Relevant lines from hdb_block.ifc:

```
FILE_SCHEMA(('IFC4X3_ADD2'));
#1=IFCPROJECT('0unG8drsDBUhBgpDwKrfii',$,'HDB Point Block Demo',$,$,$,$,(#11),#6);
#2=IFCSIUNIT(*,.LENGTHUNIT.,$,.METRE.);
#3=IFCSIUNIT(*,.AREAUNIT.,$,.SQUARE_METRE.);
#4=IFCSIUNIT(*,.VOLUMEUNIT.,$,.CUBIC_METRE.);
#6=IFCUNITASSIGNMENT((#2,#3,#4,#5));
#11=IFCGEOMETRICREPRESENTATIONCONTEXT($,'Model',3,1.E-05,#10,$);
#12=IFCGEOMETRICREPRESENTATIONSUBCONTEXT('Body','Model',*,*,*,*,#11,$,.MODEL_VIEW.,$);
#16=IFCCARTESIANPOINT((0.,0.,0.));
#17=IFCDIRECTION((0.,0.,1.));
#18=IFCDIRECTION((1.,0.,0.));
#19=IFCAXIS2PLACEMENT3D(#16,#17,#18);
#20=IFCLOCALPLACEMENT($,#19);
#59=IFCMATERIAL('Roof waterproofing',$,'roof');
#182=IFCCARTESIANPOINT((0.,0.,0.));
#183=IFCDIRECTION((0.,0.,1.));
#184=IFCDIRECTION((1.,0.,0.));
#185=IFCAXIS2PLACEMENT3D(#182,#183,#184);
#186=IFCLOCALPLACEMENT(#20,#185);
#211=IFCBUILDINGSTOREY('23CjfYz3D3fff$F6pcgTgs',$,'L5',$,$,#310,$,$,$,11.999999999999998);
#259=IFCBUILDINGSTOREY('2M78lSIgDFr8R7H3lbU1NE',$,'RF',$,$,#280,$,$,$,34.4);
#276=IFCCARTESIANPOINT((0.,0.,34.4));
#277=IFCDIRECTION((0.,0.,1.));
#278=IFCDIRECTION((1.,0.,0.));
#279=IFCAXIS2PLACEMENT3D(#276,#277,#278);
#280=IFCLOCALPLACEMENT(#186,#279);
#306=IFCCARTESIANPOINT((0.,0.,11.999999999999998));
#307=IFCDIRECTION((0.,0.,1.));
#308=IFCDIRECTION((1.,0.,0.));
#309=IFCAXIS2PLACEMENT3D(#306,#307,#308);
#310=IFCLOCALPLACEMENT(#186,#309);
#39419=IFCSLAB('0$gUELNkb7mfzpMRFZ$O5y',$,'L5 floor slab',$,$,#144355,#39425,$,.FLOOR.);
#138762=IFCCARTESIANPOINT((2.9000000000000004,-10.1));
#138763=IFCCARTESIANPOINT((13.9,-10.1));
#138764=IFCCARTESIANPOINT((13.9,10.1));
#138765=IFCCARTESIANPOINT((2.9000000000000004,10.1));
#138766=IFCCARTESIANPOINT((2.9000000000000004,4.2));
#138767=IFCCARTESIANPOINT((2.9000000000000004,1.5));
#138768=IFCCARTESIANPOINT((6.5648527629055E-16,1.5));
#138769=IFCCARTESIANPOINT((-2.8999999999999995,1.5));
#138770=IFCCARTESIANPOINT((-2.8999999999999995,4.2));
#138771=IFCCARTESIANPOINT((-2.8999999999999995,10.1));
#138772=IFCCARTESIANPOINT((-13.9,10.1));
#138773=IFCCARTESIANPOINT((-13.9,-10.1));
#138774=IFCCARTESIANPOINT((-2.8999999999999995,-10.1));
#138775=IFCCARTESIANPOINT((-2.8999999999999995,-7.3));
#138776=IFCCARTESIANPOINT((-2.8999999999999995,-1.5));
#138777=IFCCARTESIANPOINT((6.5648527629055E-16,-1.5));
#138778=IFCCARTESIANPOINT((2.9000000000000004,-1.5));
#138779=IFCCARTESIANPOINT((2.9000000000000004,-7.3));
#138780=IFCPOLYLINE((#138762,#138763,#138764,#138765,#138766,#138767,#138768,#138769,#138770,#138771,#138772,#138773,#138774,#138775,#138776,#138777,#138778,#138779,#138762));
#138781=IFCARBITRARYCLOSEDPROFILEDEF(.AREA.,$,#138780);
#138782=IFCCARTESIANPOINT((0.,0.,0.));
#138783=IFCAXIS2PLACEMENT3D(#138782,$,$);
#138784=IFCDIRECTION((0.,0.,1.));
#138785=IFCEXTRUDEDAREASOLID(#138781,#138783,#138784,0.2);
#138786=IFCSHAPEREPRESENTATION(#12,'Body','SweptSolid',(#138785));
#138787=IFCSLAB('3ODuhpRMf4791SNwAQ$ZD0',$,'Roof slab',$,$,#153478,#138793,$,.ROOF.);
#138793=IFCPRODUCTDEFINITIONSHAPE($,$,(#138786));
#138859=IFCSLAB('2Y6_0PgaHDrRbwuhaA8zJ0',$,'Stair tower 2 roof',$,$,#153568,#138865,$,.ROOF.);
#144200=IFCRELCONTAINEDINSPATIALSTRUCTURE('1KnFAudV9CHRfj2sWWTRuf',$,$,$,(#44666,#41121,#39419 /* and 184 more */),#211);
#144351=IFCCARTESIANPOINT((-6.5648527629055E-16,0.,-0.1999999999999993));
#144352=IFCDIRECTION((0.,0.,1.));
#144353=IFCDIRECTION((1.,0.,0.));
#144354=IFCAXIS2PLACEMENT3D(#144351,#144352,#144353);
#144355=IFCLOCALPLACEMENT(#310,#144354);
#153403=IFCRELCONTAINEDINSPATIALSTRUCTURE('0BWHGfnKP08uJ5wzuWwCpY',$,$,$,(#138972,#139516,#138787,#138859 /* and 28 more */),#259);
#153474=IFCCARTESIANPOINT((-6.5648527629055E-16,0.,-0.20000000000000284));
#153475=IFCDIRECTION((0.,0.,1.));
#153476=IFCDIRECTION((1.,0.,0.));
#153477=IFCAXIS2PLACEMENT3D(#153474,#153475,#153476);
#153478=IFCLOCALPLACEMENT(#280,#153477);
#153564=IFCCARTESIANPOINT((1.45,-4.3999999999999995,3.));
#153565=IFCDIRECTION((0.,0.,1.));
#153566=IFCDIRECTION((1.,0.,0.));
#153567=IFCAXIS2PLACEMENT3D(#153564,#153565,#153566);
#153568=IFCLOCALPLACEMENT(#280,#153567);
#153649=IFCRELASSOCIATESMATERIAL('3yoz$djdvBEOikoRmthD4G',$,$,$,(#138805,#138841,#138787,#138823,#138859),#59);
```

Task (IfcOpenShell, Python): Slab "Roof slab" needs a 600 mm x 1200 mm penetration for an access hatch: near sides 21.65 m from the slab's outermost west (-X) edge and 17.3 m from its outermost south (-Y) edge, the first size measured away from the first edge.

```python
import numpy as np
import ifcopenshell
import ifcopenshell.api.feature
import ifcopenshell.api.geometry
import ifcopenshell.api.root
import ifcopenshell.geom
import ifcopenshell.util.placement
import ifcopenshell.util.representation
import ifcopenshell.util.shape
import ifcopenshell.util.unit

model = ifcopenshell.open("hdb_block.ifc")
unit_scale = ifcopenshell.util.unit.calculate_unit_scale(model)
settings = ifcopenshell.geom.settings()


def volume(element):
    """Net volume in cubic metres, openings subtracted."""
    shape = ifcopenshell.geom.create_shape(settings, element)
    return ifcopenshell.util.shape.get_volume(shape.geometry)


slab = model.by_id(138787)
before = volume(slab)

# Extent in the slab's own axes, in metres. The edges named are its -X and -Y sides.
slab_shape = ifcopenshell.geom.create_shape(settings, slab)
vertices = ifcopenshell.util.shape.get_vertices(slab_shape.geometry)
x_min, y_min, bottom = vertices.min(axis=0)
top = vertices[:, 2].max()

opening = ifcopenshell.api.root.create_entity(model, ifc_class="IfcOpeningElement", name="Access hatch opening", predefined_type="OPENING")
context = ifcopenshell.util.representation.get_context(model, "Model", "Body", "MODEL_VIEW")
width, depth = 0.6, 1.2
outline = [(0.0, 0.0), (width, 0.0), (width, depth), (0.0, depth), (0.0, 0.0)]
# Overshoot both faces by 50 mm so the cut is clean.
shape = ifcopenshell.api.geometry.add_slab_representation(
    model, context=context, depth=top - bottom + 0.1, polyline=outline
)
ifcopenshell.api.geometry.assign_representation(model, product=opening, representation=shape)

matrix = ifcopenshell.util.placement.get_local_placement(slab.ObjectPlacement)
matrix[:, 3] = matrix @ np.append(np.array([x_min + 21.65, y_min + 17.3, bottom - 0.05]) / unit_scale, 1.0)
ifcopenshell.api.geometry.edit_object_placement(model, product=opening, matrix=matrix, is_si=False)
ifcopenshell.api.feature.add_feature(model, feature=opening, element=slab)

after = volume(slab)

print(f"slab volume {before:.3f} -> {after:.3f} m3")

model.write("hdb_block-out.ifc")
```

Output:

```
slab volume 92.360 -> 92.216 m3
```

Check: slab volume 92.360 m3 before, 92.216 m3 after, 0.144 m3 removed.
